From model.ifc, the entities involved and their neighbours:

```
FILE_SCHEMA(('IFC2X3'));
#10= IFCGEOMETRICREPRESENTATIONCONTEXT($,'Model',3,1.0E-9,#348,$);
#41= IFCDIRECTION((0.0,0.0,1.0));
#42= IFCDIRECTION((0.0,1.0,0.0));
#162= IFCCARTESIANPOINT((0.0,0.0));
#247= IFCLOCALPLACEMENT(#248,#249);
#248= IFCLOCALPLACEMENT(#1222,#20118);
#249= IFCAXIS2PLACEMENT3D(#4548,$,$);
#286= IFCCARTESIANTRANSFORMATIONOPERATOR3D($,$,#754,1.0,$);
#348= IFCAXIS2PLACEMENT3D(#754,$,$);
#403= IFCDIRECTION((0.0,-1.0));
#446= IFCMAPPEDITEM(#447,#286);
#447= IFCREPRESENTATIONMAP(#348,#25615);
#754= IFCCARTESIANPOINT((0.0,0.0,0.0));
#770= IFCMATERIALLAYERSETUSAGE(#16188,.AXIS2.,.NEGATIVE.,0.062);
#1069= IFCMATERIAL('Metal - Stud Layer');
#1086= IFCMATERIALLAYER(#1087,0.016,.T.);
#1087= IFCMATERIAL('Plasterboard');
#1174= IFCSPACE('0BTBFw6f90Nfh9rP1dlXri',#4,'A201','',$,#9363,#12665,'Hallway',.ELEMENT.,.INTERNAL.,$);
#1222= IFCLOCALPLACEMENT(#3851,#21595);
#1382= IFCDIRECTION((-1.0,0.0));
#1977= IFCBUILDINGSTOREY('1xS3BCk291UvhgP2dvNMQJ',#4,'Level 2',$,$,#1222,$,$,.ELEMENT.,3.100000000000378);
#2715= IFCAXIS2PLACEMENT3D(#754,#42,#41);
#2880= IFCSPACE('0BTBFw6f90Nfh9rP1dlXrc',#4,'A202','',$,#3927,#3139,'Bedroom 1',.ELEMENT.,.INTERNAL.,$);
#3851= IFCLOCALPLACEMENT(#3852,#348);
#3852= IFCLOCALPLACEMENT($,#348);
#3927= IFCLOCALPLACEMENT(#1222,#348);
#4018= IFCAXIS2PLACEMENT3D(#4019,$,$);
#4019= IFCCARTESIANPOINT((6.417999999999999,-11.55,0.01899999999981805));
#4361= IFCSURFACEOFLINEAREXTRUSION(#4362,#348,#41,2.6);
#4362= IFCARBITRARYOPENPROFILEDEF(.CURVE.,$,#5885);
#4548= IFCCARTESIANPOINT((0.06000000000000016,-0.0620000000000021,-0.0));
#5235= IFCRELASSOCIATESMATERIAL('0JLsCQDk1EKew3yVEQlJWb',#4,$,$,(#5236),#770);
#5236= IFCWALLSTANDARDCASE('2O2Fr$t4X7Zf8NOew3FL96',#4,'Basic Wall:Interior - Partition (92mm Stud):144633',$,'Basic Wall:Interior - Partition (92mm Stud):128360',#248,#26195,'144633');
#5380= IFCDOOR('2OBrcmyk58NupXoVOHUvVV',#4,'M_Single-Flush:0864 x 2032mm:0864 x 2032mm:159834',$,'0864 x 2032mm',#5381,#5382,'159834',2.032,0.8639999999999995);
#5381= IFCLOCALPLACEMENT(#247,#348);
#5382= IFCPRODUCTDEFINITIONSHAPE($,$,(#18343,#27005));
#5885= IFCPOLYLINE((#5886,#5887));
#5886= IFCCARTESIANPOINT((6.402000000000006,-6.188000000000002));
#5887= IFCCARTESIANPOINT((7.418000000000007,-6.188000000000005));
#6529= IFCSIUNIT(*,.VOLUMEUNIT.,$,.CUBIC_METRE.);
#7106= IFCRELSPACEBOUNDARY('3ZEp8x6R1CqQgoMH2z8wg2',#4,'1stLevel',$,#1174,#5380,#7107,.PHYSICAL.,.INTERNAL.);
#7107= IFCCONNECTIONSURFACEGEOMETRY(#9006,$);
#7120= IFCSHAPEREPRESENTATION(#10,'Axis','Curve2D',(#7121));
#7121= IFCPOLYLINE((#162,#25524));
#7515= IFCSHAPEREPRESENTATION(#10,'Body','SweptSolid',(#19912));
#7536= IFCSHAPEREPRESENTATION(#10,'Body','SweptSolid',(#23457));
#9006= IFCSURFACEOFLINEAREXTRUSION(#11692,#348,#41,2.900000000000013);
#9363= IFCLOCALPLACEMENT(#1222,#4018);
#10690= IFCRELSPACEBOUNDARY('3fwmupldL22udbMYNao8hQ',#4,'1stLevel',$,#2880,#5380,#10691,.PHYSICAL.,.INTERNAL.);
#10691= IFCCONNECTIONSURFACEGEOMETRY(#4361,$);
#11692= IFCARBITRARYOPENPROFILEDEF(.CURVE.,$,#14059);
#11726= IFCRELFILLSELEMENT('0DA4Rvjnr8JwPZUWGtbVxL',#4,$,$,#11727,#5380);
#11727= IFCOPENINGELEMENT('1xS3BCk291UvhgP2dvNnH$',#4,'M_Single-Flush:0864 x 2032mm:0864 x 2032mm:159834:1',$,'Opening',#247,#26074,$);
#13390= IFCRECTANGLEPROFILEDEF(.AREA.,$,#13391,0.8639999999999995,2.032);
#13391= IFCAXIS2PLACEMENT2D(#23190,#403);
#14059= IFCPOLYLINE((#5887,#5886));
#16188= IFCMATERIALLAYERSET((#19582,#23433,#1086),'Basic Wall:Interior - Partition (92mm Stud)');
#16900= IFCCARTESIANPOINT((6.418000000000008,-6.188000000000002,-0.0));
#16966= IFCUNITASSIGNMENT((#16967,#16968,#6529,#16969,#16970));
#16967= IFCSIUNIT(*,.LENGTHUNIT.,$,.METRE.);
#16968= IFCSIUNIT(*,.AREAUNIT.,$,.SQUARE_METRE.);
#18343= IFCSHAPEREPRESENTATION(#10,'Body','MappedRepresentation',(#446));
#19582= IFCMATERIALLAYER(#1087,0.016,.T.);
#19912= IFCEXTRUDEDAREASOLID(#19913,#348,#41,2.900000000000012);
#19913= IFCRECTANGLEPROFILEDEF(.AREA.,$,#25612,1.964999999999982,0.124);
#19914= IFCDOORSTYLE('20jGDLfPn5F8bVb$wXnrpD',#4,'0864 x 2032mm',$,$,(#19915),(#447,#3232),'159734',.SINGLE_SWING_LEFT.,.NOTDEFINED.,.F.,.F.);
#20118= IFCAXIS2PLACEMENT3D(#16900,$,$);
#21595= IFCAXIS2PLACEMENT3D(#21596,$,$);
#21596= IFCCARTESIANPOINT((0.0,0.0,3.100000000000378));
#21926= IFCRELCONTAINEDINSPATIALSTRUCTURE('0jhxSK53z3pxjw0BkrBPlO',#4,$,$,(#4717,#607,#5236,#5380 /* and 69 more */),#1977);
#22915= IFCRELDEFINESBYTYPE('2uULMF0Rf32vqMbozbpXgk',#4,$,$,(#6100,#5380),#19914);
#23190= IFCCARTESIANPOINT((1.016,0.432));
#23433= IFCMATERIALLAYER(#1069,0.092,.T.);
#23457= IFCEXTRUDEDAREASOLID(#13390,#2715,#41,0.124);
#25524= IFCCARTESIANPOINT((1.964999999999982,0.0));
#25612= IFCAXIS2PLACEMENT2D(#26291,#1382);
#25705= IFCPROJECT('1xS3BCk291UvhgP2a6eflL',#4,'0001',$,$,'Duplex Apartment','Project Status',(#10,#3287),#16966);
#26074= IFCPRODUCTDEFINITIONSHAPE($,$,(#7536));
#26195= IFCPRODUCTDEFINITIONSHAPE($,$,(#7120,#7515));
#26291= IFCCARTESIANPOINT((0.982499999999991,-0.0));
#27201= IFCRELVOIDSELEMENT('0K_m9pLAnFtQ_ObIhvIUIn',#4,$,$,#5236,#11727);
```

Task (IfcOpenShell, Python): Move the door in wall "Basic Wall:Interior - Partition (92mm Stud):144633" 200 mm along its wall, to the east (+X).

```python
import numpy as np
import ifcopenshell
import ifcopenshell.api.geometry
import ifcopenshell.util.placement
import ifcopenshell.util.unit

model = ifcopenshell.open("model.ifc")
unit_scale = ifcopenshell.util.unit.calculate_unit_scale(model)

door = model.by_guid("2OBrcmyk58NupXoVOHUvVV")
opening = door.FillsVoids[0].RelatingOpeningElement
wall = opening.VoidsElements[0].RelatingBuildingElement

wall_matrix = ifcopenshell.util.placement.get_local_placement(wall.ObjectPlacement)
shift = wall_matrix[:3, 0] * 0.2 / unit_scale
before = ifcopenshell.util.placement.get_local_placement(door.ObjectPlacement)[:3, 3].copy()

# The door is placed relative to its opening, so it follows when the opening moves.
matrix = ifcopenshell.util.placement.get_local_placement(opening.ObjectPlacement)
matrix[:3, 3] += shift
ifcopenshell.api.geometry.edit_object_placement(
    model, product=opening, matrix=matrix, is_si=False, should_transform_children=True
)

# Space boundary surfaces are stored in each space's coordinates; move them too.
for rel in door.ProvidesBoundaries:
    if not rel.ConnectionGeometry:
        continue
    surface = rel.ConnectionGeometry.SurfaceOnRelatingElement
    space_matrix = ifcopenshell.util.placement.get_local_placement(rel.RelatingSpace.ObjectPlacement)
    point = np.array(surface.Position.Location.Coordinates) + space_matrix[:3, :3].T @ shift
    surface.Position = model.createIfcAxis2Placement3D(
        model.createIfcCartesianPoint(point.tolist()), surface.Position.Axis, surface.Position.RefDirection
    )

after = ifcopenshell.util.placement.get_local_placement(door.ObjectPlacement)[:3, 3]
print("door moved by", (after - before).round(3) + 0.0)

model.write("model-out.ifc")
```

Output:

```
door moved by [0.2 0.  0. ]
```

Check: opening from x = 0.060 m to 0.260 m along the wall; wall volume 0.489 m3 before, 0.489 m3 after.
